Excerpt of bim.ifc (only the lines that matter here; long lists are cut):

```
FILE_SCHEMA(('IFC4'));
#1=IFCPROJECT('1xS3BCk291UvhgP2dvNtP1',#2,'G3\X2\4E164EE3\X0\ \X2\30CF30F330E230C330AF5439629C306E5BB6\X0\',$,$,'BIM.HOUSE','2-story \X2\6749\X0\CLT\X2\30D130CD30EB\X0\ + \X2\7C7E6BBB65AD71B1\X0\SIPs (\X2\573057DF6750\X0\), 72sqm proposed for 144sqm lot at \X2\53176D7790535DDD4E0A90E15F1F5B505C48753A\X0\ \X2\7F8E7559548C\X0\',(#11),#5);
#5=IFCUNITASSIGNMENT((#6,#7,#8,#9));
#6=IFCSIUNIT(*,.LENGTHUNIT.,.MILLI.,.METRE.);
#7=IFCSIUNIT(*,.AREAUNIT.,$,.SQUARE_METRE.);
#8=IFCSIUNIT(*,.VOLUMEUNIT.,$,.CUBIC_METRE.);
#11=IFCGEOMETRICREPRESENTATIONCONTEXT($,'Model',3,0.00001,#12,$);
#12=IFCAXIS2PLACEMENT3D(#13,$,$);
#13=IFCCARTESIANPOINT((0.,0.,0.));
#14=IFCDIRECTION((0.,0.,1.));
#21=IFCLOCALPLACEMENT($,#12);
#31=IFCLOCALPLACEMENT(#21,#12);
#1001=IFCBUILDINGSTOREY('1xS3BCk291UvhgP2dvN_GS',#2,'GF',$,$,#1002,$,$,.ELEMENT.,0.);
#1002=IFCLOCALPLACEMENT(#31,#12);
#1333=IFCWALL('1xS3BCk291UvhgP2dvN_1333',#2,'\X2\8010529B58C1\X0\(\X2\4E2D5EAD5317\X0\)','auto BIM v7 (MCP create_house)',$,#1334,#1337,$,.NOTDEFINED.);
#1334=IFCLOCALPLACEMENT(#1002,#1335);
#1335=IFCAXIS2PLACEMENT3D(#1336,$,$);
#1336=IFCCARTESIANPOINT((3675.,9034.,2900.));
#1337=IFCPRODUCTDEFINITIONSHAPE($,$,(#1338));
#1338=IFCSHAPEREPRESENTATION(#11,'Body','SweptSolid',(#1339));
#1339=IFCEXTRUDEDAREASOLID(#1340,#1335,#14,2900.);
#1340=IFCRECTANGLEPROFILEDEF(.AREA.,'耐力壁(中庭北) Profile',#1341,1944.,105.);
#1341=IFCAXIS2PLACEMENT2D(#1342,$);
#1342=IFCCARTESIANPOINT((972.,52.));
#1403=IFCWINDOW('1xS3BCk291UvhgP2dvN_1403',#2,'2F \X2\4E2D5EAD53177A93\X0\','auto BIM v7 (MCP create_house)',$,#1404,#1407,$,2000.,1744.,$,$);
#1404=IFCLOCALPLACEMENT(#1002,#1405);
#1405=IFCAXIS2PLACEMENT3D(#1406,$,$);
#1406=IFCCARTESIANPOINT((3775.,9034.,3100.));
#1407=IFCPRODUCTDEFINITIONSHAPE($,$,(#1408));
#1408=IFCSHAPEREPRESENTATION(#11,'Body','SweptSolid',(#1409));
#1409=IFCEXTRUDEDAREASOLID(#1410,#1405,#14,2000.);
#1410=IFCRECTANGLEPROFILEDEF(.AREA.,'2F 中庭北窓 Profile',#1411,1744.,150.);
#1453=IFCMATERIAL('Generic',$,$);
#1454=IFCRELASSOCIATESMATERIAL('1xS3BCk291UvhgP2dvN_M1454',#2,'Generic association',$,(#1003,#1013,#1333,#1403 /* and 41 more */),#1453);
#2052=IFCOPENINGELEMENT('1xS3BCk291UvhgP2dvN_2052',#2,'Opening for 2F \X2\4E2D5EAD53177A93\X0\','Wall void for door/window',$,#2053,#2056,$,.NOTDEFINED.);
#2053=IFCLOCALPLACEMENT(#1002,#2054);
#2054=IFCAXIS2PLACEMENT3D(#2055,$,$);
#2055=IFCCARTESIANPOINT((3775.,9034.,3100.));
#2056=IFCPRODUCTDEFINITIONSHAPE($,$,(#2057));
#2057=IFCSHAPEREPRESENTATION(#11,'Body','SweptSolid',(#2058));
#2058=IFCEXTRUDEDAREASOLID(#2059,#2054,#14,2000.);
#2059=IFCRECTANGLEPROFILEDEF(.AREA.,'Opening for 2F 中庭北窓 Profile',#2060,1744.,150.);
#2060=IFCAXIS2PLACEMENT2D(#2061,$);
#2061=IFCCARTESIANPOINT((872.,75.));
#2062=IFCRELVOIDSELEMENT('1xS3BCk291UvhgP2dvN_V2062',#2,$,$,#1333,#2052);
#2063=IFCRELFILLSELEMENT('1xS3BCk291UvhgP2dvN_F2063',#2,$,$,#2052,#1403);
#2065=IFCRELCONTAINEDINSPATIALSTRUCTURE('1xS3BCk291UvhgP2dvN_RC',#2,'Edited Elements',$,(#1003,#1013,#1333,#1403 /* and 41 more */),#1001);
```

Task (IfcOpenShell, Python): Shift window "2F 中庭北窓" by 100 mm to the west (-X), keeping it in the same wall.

```python
import ifcopenshell
import ifcopenshell.api.geometry
import ifcopenshell.util.placement

model = ifcopenshell.open("bim.ifc")

window = model.by_id(1403)
opening = window.FillsVoids[0].RelatingOpeningElement
wall = opening.VoidsElements[0].RelatingBuildingElement

wall_matrix = ifcopenshell.util.placement.get_local_placement(wall.ObjectPlacement)
shift = wall_matrix[:3, 0] * -100.0
before = ifcopenshell.util.placement.get_local_placement(window.ObjectPlacement)[:3, 3].copy()

# The window is not placed relative to its opening, so move both.
for product in (opening, window):
    matrix = ifcopenshell.util.placement.get_local_placement(product.ObjectPlacement)
    matrix[:3, 3] += shift
    ifcopenshell.api.geometry.edit_object_placement(model, product=product, matrix=matrix, is_si=False)

after = ifcopenshell.util.placement.get_local_placement(window.ObjectPlacement)[:3, 3]
print("window moved by", (after - before).round(3) + 0.0)

model.write("bim_edited.ifc")
```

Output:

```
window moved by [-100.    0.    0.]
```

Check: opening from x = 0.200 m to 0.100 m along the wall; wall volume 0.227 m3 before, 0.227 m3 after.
